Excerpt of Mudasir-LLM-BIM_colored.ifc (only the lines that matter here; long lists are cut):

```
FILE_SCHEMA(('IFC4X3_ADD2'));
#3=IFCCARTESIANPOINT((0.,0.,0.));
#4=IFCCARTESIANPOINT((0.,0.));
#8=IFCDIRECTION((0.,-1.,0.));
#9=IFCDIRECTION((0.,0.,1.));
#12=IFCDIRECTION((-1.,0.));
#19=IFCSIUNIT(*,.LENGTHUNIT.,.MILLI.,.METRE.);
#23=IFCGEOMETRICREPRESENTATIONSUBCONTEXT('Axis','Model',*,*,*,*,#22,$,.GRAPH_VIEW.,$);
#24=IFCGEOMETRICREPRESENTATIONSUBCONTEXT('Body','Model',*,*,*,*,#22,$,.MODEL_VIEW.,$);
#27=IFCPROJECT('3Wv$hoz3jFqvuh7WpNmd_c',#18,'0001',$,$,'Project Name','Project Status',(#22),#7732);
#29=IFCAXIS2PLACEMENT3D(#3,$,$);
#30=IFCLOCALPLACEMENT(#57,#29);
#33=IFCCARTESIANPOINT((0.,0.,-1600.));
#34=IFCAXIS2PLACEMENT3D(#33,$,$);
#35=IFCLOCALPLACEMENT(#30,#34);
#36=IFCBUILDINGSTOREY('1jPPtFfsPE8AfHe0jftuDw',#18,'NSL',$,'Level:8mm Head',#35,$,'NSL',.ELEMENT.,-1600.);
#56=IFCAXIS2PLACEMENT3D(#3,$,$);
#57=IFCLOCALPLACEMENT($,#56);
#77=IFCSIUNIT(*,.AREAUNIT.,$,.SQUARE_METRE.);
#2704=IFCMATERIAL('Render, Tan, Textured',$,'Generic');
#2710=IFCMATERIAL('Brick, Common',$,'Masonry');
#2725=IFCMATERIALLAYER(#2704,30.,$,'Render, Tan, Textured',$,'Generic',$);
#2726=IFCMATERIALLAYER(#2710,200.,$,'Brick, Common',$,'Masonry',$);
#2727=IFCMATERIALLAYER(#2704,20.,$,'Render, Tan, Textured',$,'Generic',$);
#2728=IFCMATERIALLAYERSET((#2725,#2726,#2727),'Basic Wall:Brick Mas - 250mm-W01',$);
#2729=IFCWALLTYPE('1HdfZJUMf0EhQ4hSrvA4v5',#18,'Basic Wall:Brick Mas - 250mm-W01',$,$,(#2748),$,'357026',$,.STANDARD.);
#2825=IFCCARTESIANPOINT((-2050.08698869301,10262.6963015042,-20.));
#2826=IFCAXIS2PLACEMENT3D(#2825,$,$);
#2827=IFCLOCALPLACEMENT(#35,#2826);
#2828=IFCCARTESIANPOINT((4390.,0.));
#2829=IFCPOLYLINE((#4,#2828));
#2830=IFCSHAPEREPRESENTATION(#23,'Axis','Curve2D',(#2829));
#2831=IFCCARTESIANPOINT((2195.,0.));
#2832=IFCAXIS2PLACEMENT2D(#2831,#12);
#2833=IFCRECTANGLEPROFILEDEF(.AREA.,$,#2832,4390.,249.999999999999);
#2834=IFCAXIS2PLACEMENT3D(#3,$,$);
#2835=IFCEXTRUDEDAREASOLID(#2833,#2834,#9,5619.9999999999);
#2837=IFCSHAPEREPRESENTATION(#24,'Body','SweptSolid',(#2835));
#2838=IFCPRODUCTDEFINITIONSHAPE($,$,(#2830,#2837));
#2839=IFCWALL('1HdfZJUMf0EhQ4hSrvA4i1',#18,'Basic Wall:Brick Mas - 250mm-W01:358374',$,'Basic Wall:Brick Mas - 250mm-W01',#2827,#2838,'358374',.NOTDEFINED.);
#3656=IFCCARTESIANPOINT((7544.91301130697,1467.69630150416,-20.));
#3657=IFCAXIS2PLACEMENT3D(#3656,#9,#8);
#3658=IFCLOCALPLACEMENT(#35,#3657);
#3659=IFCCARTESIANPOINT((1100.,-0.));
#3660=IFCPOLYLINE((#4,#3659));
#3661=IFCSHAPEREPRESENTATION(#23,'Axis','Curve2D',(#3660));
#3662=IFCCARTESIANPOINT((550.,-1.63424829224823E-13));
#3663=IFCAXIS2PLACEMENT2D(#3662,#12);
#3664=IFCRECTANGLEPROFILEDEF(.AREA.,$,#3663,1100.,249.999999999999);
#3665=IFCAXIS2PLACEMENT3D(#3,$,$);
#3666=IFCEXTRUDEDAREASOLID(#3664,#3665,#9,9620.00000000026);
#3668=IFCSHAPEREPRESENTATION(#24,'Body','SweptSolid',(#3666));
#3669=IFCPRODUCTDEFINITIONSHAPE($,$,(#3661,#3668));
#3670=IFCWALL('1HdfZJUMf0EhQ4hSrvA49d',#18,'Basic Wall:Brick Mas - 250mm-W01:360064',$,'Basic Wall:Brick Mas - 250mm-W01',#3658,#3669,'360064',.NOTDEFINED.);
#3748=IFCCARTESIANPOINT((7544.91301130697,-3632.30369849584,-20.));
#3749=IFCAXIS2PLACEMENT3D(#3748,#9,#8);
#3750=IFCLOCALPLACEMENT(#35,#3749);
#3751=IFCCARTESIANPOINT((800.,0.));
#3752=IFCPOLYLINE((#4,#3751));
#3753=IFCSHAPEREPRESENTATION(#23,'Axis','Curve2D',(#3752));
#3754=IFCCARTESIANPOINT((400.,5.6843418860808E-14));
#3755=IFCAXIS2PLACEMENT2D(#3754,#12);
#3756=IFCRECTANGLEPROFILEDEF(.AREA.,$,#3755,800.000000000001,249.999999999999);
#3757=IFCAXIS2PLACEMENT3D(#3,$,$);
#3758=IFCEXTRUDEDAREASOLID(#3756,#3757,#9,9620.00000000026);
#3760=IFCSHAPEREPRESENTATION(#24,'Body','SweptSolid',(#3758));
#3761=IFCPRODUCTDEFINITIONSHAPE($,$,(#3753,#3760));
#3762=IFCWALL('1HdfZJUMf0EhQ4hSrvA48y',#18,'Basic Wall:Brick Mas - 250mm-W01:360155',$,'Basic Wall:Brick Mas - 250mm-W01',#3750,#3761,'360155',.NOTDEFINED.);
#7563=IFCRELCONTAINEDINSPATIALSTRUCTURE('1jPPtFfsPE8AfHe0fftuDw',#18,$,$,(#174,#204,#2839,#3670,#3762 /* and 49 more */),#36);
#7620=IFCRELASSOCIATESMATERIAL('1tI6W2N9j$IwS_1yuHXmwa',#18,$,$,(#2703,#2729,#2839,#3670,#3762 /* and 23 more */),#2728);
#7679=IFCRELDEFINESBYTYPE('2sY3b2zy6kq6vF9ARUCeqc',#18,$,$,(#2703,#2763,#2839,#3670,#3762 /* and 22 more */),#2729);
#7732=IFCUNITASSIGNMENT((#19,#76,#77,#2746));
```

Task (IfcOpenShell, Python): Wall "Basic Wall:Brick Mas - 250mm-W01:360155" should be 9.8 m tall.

```python
import ifcopenshell
import ifcopenshell.geom
import ifcopenshell.util.representation
import ifcopenshell.util.shape

model = ifcopenshell.open("Mudasir-LLM-BIM_colored.ifc")
settings = ifcopenshell.geom.settings()


def volume(element):
    """Net volume in cubic metres, openings subtracted."""
    shape = ifcopenshell.geom.create_shape(settings, element)
    return ifcopenshell.util.shape.get_volume(shape.geometry)


wall = model.by_guid("1HdfZJUMf0EhQ4hSrvA48y")
before = volume(wall)

body = ifcopenshell.util.representation.get_representation(wall, "Model", "Body")
solid = body.Items[0]
old_height = solid.Depth
solid.Depth = 9800.0
after = volume(wall)

print(f"height {old_height:g} -> {solid.Depth:g}, volume {before:.3f} -> {after:.3f} m3")

model.write("Mudasir-LLM-BIM_colored_v2.ifc")
```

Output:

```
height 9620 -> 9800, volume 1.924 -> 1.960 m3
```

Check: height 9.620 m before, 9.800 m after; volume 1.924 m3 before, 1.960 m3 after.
